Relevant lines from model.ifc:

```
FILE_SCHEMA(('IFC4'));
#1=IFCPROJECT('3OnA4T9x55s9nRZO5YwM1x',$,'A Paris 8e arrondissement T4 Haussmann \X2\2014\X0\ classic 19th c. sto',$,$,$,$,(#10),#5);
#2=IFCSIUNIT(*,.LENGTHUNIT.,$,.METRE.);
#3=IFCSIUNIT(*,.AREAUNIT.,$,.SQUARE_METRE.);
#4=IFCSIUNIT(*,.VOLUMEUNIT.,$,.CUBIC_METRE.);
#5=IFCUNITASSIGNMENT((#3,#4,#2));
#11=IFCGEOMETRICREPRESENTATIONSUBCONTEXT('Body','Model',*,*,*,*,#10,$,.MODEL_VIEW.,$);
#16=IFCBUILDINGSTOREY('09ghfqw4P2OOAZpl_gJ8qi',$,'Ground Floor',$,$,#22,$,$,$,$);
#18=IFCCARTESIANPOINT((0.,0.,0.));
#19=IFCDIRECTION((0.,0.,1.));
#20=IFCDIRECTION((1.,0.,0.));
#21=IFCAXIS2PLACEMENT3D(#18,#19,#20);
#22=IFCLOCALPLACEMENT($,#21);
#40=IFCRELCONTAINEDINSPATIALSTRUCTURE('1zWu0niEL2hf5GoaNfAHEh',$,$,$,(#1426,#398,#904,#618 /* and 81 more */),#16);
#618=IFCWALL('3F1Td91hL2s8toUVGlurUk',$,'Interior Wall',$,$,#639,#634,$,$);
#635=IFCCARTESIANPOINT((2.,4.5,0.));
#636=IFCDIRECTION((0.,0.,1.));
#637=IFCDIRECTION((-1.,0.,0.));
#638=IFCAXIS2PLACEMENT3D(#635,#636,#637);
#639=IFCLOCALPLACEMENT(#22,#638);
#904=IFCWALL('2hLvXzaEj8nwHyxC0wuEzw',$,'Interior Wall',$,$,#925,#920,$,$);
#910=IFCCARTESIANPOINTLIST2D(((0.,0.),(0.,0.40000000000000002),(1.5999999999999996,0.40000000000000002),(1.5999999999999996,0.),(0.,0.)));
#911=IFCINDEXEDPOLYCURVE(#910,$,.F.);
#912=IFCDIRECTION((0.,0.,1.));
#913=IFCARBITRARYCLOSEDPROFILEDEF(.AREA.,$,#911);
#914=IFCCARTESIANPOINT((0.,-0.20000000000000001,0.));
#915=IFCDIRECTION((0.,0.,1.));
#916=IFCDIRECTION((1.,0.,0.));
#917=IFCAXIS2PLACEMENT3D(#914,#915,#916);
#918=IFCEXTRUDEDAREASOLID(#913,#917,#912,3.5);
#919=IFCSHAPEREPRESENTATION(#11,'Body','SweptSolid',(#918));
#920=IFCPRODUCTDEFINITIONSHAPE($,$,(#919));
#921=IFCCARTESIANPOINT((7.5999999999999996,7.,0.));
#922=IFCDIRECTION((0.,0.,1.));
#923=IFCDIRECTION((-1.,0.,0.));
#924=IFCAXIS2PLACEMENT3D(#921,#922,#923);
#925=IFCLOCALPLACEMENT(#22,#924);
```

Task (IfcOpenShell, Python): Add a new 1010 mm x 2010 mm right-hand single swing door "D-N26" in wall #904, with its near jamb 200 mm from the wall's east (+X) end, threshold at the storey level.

```python
import numpy as np
import ifcopenshell
import ifcopenshell.api.feature
import ifcopenshell.api.geometry
import ifcopenshell.api.root
import ifcopenshell.api.spatial
import ifcopenshell.geom
import ifcopenshell.util.element
import ifcopenshell.util.placement
import ifcopenshell.util.representation
import ifcopenshell.util.shape
import ifcopenshell.util.unit

model = ifcopenshell.open("model.ifc")
unit_scale = ifcopenshell.util.unit.calculate_unit_scale(model)
settings = ifcopenshell.geom.settings()


def volume(element):
    """Net volume in cubic metres, openings subtracted."""
    shape = ifcopenshell.geom.create_shape(settings, element)
    return ifcopenshell.util.shape.get_volume(shape.geometry)


wall = model.by_guid("2hLvXzaEj8nwHyxC0wuEzw")
storey = ifcopenshell.util.element.get_container(wall, ifc_class="IfcBuildingStorey")
context = ifcopenshell.util.representation.get_context(model, "Model", "Body", "MODEL_VIEW")
before = volume(wall)

width, height, from_end, sill = 1.01, 2.01, 0.2, 0.0  # metres

# The wall runs along its own X axis, and the end named is its -X end.
wall_shape = ifcopenshell.geom.create_shape(settings, wall)
x, y, z = ifcopenshell.util.shape.get_vertices(wall_shape.geometry).T
start = x.min() + from_end
face, thickness = float(y.min()), float(y.max() - y.min())
wall_matrix = ifcopenshell.util.placement.get_local_placement(wall.ObjectPlacement)
level = ifcopenshell.util.placement.get_local_placement(storey.ObjectPlacement)[2, 3]


def in_wall(x, y):
    """Placement at x, y metres in the wall's axes, at sill height."""
    matrix = wall_matrix.copy()
    matrix[:, 3] = wall_matrix @ np.array([x / unit_scale, y / unit_scale, 0.0, 1.0])
    matrix[2, 3] = level + sill / unit_scale
    return matrix


# Opening: a box that overshoots both wall faces by 50 mm.
opening = ifcopenshell.api.root.create_entity(model, ifc_class="IfcOpeningElement", predefined_type="OPENING")
box = ifcopenshell.api.geometry.add_wall_representation(
    model, context=context, length=width, height=height, thickness=thickness + 0.1
)
ifcopenshell.api.geometry.assign_representation(model, product=opening, representation=box)
ifcopenshell.api.geometry.edit_object_placement(model, product=opening, matrix=in_wall(start, face - 0.05), is_si=False)
ifcopenshell.api.feature.add_feature(model, feature=opening, element=wall)

door = ifcopenshell.api.root.create_entity(model, ifc_class="IfcDoor", name="D-N26", predefined_type="DOOR")
door.OverallWidth, door.OverallHeight = width / unit_scale, height / unit_scale
door.OperationType = "SINGLE_SWING_RIGHT"
body = ifcopenshell.api.geometry.add_door_representation(
    model,
    context=context,
    overall_width=door.OverallWidth,
    overall_height=door.OverallHeight,
    operation_type="SINGLE_SWING_RIGHT",
    lining_properties={"LiningDepth": thickness / unit_scale, "ThresholdDepth": thickness / unit_scale},
)
ifcopenshell.api.geometry.assign_representation(model, product=door, representation=body)
ifcopenshell.api.spatial.assign_container(model, products=[door], relating_structure=storey)
ifcopenshell.api.feature.add_filling(model, opening=opening, element=door)

# The lining spans the wall, so the door starts at the wall face.
ifcopenshell.api.geometry.edit_object_placement(model, product=door, matrix=in_wall(start, face), is_si=False)

after = volume(wall)

print(f"wall volume {before:.3f} -> {after:.3f} m3")

model.write("model-out.ifc")
```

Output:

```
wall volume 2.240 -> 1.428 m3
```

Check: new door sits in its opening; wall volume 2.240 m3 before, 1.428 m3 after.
